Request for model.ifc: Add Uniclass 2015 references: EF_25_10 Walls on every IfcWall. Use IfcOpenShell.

First a look at what the model holds.

```python
import ifcopenshell

model = ifcopenshell.open("model.ifc")
print(model.schema)
print("classifications:", [c.Name for c in model.by_type("IfcClassification")])
for ifc_class in ("IfcDoor", "IfcRoof", "IfcStair", "IfcWall", "IfcWindow"):
    print(ifc_class, len(model.by_type(ifc_class)))
```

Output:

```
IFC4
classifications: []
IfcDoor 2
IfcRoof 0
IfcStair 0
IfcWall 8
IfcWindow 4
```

```python
import ifcopenshell
import ifcopenshell.api.classification

model = ifcopenshell.open("model.ifc")

system = ifcopenshell.api.classification.add_classification(model, classification="Uniclass 2015")

codes = {
    "IfcWall": ("EF_25_10", "Walls"),
}
for ifc_class, (code, name) in codes.items():
    products = model.by_type(ifc_class)
    ifcopenshell.api.classification.add_reference(
        model, products=products, classification=system, identification=code, name=name
    )
    print(code, len(products))

model.write("model_v2.ifc")
```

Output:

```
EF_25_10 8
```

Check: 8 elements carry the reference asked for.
